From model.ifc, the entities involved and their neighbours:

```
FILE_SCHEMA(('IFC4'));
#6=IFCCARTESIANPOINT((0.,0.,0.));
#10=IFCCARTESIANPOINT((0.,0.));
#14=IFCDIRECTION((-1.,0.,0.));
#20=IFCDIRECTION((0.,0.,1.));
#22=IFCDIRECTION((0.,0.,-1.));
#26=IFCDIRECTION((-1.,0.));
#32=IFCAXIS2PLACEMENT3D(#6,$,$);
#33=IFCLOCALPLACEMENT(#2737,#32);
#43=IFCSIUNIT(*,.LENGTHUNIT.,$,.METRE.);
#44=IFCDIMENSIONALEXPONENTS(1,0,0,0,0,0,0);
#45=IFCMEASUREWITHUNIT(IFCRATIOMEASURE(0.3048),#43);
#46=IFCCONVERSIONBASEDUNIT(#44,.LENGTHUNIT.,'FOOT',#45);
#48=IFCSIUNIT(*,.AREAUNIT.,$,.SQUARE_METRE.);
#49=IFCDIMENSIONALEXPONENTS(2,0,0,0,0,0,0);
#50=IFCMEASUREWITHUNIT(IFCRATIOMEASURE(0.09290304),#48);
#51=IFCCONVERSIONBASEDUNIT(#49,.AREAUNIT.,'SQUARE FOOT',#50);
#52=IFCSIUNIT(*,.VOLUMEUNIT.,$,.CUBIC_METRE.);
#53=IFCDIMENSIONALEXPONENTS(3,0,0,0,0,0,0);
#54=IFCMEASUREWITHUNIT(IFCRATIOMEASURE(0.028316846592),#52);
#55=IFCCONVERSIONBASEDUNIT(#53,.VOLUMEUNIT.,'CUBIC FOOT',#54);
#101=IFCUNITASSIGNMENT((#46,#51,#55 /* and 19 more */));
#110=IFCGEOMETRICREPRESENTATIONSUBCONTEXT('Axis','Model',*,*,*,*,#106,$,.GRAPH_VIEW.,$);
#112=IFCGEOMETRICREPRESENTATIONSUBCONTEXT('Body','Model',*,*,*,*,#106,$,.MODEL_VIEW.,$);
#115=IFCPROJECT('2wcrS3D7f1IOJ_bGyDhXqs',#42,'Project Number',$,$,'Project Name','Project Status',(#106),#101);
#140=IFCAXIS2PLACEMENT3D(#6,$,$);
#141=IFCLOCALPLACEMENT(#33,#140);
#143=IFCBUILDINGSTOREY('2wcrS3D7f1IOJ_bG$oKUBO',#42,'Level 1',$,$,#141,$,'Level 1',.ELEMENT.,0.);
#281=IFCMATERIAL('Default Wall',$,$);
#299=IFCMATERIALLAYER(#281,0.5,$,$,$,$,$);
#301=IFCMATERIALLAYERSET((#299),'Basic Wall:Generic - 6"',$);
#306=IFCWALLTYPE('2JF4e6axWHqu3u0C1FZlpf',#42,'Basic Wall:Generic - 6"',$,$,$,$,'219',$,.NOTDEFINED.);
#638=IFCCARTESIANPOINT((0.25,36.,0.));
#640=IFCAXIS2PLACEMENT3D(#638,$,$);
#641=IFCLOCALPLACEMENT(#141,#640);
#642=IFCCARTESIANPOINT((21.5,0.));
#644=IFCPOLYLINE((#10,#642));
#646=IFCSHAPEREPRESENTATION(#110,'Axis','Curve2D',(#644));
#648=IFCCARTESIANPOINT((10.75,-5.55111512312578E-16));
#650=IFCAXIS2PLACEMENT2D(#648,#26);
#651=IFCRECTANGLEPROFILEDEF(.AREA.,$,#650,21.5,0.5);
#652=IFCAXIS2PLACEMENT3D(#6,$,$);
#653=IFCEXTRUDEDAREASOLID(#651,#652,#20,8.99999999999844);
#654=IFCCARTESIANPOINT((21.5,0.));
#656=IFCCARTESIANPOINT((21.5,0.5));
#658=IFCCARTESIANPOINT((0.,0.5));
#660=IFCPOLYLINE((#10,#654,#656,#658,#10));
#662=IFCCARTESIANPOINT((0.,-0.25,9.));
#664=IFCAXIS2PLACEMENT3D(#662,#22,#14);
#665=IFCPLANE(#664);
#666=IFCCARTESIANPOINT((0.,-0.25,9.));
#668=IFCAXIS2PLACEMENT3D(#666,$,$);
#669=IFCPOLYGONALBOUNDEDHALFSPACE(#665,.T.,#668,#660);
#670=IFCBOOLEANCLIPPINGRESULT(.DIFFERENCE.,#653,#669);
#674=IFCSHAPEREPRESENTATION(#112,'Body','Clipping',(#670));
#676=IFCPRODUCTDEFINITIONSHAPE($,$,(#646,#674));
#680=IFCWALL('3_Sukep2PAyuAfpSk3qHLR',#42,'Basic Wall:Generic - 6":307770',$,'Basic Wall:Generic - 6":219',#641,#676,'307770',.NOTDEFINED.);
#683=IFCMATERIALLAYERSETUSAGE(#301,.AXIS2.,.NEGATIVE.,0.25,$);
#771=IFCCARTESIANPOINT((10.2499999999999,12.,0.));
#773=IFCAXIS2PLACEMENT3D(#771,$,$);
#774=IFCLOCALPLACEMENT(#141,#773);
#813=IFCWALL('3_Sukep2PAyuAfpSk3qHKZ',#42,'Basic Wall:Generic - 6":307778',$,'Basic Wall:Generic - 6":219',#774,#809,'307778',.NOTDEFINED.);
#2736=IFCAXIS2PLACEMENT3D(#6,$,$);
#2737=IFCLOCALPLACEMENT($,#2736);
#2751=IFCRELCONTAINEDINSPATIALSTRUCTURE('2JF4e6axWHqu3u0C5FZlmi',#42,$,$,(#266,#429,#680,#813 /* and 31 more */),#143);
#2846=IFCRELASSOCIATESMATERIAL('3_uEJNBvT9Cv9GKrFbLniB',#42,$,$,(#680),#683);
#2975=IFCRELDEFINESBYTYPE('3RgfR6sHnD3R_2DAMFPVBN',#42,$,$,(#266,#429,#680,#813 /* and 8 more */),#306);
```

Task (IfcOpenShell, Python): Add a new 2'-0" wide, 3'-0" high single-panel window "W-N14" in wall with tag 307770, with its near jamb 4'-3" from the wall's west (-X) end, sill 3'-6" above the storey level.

```python
import numpy as np
import ifcopenshell
import ifcopenshell.api.feature
import ifcopenshell.api.geometry
import ifcopenshell.api.root
import ifcopenshell.api.spatial
import ifcopenshell.geom
import ifcopenshell.util.element
import ifcopenshell.util.placement
import ifcopenshell.util.representation
import ifcopenshell.util.shape
import ifcopenshell.util.unit

model = ifcopenshell.open("model.ifc")
unit_scale = ifcopenshell.util.unit.calculate_unit_scale(model)
settings = ifcopenshell.geom.settings()


def volume(element):
    """Net volume in cubic metres, openings subtracted."""
    shape = ifcopenshell.geom.create_shape(settings, element)
    return ifcopenshell.util.shape.get_volume(shape.geometry)


wall = model.by_id(680)
storey = ifcopenshell.util.element.get_container(wall, ifc_class="IfcBuildingStorey")
context = ifcopenshell.util.representation.get_context(model, "Model", "Body", "MODEL_VIEW")
before = volume(wall)

width, height, from_end, sill = 0.6096, 0.9144, 1.2954, 1.0668  # metres

# The wall runs along its own X axis, and the end named is its -X end.
wall_shape = ifcopenshell.geom.create_shape(settings, wall)
x, y, z = ifcopenshell.util.shape.get_vertices(wall_shape.geometry).T
start = x.min() + from_end
face, thickness = float(y.min()), float(y.max() - y.min())
wall_matrix = ifcopenshell.util.placement.get_local_placement(wall.ObjectPlacement)
level = ifcopenshell.util.placement.get_local_placement(storey.ObjectPlacement)[2, 3]


def in_wall(x, y):
    """Placement at x, y metres in the wall's axes, at sill height."""
    matrix = wall_matrix.copy()
    matrix[:, 3] = wall_matrix @ np.array([x / unit_scale, y / unit_scale, 0.0, 1.0])
    matrix[2, 3] = level + sill / unit_scale
    return matrix


# Opening: a box that overshoots both wall faces by 50 mm.
opening = ifcopenshell.api.root.create_entity(model, ifc_class="IfcOpeningElement", predefined_type="OPENING")
box = ifcopenshell.api.geometry.add_wall_representation(
    model, context=context, length=width, height=height, thickness=thickness + 0.1
)
ifcopenshell.api.geometry.assign_representation(model, product=opening, representation=box)
ifcopenshell.api.geometry.edit_object_placement(model, product=opening, matrix=in_wall(start, face - 0.05), is_si=False)
ifcopenshell.api.feature.add_feature(model, feature=opening, element=wall)

window = ifcopenshell.api.root.create_entity(model, ifc_class="IfcWindow", name="W-N14", predefined_type="WINDOW")
window.OverallWidth, window.OverallHeight = width / unit_scale, height / unit_scale
window.PartitioningType = "SINGLE_PANEL"
body = ifcopenshell.api.geometry.add_window_representation(
    model,
    context=context,
    overall_width=window.OverallWidth,
    overall_height=window.OverallHeight,
    partition_type="SINGLE_PANEL",
)
ifcopenshell.api.geometry.assign_representation(model, product=window, representation=body)
ifcopenshell.api.spatial.assign_container(model, products=[window], relating_structure=storey)
ifcopenshell.api.feature.add_filling(model, opening=opening, element=window)

# Centre the window in the wall's thickness.
ifcopenshell.api.geometry.edit_object_placement(model, product=window, matrix=in_wall(start, face), is_si=False)
window_shape = ifcopenshell.geom.create_shape(settings, window)
depth = ifcopenshell.util.shape.get_vertices(window_shape.geometry)[:, 1]
offset = face + thickness / 2 - (depth.min() + depth.max()) / 2
ifcopenshell.api.geometry.edit_object_placement(model, product=window, matrix=in_wall(start, offset), is_si=False)

after = volume(wall)

print(f"wall volume {before:.3f} -> {after:.3f} m3")

model.write("model_v2.ifc")
```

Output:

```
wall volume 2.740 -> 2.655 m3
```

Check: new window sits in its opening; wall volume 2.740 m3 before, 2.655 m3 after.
